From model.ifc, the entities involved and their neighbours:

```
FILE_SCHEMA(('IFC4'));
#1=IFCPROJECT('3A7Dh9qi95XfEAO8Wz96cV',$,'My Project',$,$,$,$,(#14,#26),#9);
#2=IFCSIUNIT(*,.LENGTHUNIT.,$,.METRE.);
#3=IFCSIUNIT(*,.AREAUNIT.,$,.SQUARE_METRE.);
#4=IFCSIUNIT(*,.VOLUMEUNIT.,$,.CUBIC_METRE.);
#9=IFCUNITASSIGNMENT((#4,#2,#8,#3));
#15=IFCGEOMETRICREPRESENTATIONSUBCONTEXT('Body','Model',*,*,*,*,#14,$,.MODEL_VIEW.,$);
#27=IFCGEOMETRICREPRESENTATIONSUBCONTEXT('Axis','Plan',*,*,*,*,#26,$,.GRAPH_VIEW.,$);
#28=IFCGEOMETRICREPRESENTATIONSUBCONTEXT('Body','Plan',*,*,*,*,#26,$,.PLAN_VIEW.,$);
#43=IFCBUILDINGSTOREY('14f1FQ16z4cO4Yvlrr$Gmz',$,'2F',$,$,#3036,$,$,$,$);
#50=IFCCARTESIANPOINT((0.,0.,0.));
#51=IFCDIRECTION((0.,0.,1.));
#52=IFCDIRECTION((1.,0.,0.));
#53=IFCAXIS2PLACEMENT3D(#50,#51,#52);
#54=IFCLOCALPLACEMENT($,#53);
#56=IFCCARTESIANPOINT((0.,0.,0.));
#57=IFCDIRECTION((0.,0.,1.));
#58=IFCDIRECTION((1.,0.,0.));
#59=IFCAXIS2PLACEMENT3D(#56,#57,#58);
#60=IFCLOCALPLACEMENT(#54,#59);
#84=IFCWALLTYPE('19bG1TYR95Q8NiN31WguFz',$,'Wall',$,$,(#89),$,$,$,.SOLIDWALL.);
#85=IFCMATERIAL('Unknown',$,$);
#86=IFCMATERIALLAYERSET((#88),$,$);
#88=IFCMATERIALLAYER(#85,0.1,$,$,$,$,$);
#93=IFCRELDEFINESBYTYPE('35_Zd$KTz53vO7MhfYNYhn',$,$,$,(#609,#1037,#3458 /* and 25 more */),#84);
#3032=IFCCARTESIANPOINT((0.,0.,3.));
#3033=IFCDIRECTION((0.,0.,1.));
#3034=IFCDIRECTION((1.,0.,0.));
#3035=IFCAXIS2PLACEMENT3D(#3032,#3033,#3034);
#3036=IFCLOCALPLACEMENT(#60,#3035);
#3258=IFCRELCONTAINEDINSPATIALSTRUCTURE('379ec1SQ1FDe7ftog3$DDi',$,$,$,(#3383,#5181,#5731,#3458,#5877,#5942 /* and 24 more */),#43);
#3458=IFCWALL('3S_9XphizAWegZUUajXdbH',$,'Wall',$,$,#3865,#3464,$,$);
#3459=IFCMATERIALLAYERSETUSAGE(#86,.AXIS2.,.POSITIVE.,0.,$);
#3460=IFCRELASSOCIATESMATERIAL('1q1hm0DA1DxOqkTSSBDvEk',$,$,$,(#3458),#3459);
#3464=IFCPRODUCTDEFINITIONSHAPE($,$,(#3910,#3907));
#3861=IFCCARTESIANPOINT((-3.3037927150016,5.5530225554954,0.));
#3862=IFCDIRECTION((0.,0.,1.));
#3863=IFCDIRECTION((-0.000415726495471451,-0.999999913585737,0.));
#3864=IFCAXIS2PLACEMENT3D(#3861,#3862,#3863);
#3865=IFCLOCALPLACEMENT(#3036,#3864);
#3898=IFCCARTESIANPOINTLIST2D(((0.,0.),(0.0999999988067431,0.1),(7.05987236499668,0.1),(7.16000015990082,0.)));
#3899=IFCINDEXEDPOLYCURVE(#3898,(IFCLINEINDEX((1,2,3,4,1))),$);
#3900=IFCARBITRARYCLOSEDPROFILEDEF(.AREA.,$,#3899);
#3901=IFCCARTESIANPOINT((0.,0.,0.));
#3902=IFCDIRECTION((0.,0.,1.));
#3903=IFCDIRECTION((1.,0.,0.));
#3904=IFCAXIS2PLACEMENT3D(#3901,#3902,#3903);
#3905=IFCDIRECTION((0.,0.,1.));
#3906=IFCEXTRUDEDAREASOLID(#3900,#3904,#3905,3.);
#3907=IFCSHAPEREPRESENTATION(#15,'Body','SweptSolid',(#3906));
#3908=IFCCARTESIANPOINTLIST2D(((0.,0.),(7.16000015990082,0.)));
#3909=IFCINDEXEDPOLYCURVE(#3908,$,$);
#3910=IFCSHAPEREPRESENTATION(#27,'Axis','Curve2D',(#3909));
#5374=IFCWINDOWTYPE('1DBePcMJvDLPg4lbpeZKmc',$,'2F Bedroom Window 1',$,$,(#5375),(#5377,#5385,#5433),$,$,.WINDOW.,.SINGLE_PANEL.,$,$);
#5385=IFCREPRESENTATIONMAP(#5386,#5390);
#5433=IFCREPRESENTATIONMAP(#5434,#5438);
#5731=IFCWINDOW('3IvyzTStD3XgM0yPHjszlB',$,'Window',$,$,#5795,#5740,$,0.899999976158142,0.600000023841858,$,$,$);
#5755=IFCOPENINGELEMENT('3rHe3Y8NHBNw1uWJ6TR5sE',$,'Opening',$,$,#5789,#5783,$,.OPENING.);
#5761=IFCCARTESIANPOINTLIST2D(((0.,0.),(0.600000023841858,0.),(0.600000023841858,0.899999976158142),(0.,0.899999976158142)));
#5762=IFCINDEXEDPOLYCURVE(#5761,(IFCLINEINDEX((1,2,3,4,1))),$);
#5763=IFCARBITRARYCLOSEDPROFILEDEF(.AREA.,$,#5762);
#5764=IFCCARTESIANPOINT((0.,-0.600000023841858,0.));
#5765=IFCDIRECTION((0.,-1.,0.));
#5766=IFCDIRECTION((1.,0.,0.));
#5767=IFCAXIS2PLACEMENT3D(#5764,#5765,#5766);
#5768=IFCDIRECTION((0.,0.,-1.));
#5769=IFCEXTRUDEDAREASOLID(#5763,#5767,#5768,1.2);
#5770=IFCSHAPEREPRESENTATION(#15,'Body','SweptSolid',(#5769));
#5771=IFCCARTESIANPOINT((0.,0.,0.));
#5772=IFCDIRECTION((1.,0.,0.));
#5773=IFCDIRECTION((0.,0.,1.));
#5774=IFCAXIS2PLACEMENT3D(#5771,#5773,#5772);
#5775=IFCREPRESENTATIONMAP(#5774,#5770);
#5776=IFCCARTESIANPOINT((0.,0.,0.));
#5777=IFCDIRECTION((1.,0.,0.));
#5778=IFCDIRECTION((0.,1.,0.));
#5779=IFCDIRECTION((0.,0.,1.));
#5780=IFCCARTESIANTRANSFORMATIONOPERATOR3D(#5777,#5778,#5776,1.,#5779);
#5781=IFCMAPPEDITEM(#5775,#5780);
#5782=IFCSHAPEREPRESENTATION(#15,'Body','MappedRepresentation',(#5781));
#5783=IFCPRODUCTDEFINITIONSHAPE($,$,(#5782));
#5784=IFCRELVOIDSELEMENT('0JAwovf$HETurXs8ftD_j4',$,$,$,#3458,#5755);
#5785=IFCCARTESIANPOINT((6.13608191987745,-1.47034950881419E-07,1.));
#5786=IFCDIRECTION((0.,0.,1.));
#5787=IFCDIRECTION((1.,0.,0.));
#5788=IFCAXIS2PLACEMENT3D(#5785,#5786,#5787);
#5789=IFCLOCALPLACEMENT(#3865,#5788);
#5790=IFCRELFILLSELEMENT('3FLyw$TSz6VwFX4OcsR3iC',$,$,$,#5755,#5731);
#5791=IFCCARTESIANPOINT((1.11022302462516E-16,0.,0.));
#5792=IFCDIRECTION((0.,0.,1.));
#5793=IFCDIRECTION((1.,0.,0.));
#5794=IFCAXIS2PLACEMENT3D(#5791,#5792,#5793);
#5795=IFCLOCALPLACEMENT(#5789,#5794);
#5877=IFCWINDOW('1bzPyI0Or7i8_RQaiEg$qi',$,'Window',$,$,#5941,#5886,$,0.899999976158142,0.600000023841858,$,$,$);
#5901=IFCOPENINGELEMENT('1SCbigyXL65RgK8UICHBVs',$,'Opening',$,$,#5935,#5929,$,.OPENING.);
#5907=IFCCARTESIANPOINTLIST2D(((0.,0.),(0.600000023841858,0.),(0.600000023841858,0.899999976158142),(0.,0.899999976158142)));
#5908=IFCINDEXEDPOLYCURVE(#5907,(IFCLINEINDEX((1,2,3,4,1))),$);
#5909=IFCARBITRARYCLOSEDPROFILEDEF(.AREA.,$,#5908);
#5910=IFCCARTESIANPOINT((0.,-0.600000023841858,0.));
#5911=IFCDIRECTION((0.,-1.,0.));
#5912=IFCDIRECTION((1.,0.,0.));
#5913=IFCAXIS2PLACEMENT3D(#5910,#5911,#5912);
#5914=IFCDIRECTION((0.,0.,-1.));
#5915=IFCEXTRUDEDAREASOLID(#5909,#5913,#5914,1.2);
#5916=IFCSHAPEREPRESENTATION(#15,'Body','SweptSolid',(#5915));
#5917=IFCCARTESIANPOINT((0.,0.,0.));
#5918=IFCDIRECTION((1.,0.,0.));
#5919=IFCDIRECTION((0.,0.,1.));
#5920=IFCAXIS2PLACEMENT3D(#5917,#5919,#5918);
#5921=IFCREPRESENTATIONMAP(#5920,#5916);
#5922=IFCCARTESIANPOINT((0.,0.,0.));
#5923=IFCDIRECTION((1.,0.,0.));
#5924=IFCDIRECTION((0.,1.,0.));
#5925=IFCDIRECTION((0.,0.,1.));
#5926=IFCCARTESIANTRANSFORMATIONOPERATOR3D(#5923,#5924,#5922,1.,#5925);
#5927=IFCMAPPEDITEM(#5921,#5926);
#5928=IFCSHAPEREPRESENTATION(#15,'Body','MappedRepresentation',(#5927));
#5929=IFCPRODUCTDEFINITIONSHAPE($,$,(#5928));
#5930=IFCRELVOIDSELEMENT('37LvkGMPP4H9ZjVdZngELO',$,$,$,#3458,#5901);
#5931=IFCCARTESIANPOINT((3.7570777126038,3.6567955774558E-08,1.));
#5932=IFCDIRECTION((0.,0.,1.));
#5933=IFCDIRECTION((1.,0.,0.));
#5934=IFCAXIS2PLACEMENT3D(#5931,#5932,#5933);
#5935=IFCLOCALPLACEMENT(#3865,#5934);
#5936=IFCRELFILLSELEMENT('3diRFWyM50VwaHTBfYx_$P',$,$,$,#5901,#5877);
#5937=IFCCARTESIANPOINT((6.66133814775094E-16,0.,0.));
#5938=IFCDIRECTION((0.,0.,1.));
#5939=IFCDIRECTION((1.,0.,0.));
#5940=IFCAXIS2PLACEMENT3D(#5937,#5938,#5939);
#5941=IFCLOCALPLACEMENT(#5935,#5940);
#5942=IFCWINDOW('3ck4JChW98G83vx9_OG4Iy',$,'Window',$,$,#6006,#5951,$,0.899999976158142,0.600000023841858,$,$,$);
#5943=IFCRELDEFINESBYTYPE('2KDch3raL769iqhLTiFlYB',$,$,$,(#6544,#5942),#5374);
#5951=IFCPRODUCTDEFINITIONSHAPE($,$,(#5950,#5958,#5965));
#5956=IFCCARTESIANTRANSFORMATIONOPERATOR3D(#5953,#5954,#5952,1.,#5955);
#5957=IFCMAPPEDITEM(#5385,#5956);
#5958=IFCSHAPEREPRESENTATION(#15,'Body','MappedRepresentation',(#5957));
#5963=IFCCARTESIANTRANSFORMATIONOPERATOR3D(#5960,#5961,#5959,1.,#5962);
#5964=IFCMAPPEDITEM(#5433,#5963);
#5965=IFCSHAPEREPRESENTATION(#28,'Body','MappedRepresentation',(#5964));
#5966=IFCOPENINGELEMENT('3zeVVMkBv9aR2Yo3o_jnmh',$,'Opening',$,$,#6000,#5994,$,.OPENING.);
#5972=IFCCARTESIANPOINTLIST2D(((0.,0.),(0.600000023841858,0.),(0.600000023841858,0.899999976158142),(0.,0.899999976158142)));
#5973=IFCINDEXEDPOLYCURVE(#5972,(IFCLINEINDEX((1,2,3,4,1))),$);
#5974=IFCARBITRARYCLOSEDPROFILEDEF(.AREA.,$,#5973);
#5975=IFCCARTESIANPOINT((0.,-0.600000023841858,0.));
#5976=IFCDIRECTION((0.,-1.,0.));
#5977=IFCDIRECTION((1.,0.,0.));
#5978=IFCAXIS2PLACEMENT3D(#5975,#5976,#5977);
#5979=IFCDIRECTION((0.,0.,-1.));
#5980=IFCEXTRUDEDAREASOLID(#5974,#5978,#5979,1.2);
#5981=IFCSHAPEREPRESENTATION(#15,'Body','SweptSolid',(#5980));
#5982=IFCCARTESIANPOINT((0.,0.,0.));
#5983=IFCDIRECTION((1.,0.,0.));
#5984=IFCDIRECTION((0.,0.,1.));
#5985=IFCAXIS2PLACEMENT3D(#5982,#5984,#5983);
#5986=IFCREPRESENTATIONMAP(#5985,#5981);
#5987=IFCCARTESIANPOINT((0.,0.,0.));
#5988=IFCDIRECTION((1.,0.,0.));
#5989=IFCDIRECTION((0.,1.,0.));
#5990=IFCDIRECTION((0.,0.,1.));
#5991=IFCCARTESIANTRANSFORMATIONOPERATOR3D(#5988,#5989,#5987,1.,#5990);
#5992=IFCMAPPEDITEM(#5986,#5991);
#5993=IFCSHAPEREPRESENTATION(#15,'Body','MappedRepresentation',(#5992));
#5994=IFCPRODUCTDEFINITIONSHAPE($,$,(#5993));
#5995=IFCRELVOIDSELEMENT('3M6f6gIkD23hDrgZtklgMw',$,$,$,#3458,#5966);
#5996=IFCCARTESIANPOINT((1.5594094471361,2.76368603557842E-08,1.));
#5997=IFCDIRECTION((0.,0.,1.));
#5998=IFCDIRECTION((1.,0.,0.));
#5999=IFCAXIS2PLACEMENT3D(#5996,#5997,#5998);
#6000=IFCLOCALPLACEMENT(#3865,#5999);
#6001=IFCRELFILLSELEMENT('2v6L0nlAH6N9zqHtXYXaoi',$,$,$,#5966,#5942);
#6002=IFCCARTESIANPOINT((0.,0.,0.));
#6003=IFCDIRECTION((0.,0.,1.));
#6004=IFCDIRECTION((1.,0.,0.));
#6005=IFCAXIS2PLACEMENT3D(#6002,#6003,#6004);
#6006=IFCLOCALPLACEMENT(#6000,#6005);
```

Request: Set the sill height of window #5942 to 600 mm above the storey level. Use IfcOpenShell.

```python
import numpy as np
import ifcopenshell
import ifcopenshell.api.geometry
import ifcopenshell.geom
import ifcopenshell.util.element
import ifcopenshell.util.placement
import ifcopenshell.util.shape
import ifcopenshell.util.unit

model = ifcopenshell.open("model.ifc")
unit_scale = ifcopenshell.util.unit.calculate_unit_scale(model)

window = model.by_guid("3ck4JChW98G83vx9_OG4Iy")
opening = window.FillsVoids[0].RelatingOpeningElement
storey = ifcopenshell.util.element.get_container(window, ifc_class="IfcBuildingStorey")
level = ifcopenshell.util.placement.get_local_placement(storey.ObjectPlacement)[2, 3]

# The opening's origin need not be at the sill, so measure its lowest point.
shape = ifcopenshell.geom.create_shape(ifcopenshell.geom.settings(), opening)
bottom = ifcopenshell.util.shape.get_shape_bottom_elevation(shape, shape.geometry) / unit_scale
dz = level + 0.6 / unit_scale - bottom

shift = np.array([0.0, 0.0, dz])
# The window is placed relative to its opening, so it follows when the opening moves.
matrix = ifcopenshell.util.placement.get_local_placement(opening.ObjectPlacement)
matrix[:3, 3] += shift
ifcopenshell.api.geometry.edit_object_placement(
    model, product=opening, matrix=matrix, is_si=False, should_transform_children=True
)

print(f"moved by {dz * unit_scale:+.3f} m")

model.write("model-out.ifc")
```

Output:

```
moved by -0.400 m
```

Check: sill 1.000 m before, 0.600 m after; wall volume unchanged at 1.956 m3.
